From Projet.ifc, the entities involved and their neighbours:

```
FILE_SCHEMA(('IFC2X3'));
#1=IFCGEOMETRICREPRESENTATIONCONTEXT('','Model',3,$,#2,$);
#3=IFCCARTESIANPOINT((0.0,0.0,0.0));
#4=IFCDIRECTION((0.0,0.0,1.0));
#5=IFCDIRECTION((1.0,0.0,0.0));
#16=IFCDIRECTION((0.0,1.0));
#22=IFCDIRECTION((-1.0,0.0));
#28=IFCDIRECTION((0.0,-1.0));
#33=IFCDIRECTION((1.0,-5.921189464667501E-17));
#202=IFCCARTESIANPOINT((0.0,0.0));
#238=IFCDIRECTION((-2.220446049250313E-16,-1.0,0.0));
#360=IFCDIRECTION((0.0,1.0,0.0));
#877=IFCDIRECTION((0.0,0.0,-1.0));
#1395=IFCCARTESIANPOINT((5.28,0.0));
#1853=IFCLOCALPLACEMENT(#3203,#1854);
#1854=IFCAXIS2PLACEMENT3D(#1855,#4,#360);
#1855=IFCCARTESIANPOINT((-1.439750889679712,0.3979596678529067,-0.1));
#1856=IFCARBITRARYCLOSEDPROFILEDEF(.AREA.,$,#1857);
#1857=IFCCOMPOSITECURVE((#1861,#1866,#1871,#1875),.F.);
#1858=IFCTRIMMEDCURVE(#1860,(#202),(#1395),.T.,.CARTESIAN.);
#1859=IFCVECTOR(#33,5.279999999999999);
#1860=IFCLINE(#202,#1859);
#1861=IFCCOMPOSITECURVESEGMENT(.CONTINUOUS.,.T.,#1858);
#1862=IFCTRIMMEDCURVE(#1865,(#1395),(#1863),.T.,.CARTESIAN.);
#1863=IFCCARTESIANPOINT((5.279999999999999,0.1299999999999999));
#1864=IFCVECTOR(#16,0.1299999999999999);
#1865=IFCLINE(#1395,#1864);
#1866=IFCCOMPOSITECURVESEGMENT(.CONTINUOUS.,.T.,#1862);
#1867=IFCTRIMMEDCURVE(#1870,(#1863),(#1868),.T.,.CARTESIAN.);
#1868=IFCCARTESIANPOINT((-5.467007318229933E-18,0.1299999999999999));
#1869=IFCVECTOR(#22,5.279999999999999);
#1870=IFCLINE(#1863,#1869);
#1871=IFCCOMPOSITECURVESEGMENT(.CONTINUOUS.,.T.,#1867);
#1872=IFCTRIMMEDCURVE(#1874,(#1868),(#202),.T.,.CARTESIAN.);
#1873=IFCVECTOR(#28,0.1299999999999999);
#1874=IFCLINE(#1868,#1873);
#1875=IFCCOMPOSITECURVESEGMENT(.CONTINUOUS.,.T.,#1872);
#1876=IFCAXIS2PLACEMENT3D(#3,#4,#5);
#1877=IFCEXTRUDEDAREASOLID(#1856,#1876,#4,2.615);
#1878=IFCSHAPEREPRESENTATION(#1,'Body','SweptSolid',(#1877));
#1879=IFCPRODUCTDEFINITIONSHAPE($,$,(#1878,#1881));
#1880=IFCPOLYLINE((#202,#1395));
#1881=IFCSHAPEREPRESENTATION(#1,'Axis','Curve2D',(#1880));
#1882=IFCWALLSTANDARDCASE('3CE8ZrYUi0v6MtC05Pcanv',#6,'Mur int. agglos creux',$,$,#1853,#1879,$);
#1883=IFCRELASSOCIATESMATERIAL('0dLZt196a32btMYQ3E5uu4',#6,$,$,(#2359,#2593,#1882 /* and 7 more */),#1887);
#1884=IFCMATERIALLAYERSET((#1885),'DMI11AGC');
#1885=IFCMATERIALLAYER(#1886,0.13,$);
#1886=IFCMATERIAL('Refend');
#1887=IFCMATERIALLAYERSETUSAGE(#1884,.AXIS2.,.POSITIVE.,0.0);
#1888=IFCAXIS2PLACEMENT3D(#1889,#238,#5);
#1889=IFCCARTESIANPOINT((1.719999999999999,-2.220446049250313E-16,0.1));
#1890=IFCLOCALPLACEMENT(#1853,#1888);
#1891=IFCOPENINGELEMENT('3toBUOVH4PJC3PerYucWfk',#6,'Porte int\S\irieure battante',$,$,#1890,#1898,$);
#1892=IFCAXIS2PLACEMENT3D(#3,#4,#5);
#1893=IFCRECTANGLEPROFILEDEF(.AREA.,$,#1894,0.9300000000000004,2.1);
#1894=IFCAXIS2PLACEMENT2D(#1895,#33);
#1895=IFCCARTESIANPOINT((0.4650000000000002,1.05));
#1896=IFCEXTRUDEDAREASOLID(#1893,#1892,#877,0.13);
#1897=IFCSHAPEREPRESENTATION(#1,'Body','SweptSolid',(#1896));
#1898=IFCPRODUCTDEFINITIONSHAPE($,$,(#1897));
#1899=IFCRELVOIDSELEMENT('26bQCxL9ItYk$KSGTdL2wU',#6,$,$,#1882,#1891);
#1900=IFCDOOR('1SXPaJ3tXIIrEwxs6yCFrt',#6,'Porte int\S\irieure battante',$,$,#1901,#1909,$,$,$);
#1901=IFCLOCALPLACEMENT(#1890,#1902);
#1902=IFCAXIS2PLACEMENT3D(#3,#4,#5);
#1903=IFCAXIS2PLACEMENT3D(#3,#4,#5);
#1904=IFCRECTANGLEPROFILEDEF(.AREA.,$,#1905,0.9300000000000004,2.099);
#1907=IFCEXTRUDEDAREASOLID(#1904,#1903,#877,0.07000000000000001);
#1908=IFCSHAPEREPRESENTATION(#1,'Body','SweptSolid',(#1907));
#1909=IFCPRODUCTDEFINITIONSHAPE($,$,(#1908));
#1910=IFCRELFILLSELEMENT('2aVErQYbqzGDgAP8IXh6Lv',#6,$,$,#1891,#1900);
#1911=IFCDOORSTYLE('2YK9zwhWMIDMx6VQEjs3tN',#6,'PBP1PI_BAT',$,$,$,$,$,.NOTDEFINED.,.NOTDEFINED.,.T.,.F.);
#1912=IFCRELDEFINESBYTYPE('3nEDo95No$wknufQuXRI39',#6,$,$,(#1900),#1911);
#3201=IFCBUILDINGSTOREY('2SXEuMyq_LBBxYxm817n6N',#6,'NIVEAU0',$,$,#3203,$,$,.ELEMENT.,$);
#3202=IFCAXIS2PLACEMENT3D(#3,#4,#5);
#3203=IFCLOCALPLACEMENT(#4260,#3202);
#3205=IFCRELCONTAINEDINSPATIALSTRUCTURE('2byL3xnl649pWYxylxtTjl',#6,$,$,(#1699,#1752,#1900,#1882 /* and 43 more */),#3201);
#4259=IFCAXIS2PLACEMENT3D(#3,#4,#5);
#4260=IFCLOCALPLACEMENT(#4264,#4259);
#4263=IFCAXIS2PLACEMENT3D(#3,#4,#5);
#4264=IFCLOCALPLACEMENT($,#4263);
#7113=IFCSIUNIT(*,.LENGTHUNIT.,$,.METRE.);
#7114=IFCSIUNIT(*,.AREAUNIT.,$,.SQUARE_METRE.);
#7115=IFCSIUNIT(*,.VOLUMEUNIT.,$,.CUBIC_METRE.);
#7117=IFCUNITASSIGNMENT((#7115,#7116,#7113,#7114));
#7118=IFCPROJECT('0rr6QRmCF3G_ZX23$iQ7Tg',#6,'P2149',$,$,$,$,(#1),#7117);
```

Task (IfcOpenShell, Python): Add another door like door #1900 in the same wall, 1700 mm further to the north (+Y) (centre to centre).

```python
import ifcopenshell
import ifcopenshell.api.feature
import ifcopenshell.api.geometry
import ifcopenshell.api.root
import ifcopenshell.geom
import ifcopenshell.util.element
import ifcopenshell.util.placement
import ifcopenshell.util.shape

model = ifcopenshell.open("Projet.ifc")
settings = ifcopenshell.geom.settings()


def volume(element):
    """Net volume in cubic metres, openings subtracted."""
    shape = ifcopenshell.geom.create_shape(settings, element)
    return ifcopenshell.util.shape.get_volume(shape.geometry)


door = model.by_guid("1SXPaJ3tXIIrEwxs6yCFrt")
opening = door.FillsVoids[0].RelatingOpeningElement
wall = opening.VoidsElements[0].RelatingBuildingElement
before = volume(wall)
shift = ifcopenshell.util.placement.get_local_placement(wall.ObjectPlacement)[:3, 0] * 1.7

# copy_class copies the void relationship, type, container and properties, but no geometry.
new_opening = ifcopenshell.api.root.copy_class(model, product=opening)
new_opening.Representation = ifcopenshell.util.element.copy_deep(
    model, opening.Representation, exclude=["IfcGeometricRepresentationContext", "IfcRepresentationMap"]
)
new_door = ifcopenshell.api.root.copy_class(model, product=door)
new_door.Representation = ifcopenshell.util.element.copy_deep(
    model, door.Representation, exclude=["IfcGeometricRepresentationContext", "IfcRepresentationMap"]
)
fills = ifcopenshell.api.feature.add_filling(model, opening=new_opening, element=new_door)
fills.OwnerHistory = new_door.OwnerHistory  # required in IFC2X3

for old, new in ((opening, new_opening), (door, new_door)):
    matrix = ifcopenshell.util.placement.get_local_placement(old.ObjectPlacement)
    matrix[:3, 3] += shift
    ifcopenshell.api.geometry.edit_object_placement(model, product=new, matrix=matrix, is_si=False)

after = volume(wall)

print(f"wall volume {before:.3f} -> {after:.3f} m3")

model.write("Projet_v2.ifc")
```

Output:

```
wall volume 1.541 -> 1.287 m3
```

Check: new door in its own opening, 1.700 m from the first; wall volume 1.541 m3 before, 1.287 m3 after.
